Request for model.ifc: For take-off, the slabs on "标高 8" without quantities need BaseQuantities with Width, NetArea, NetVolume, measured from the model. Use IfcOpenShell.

First a look at what the model holds.

```python
import ifcopenshell
import ifcopenshell.util.element
import ifcopenshell.util.unit

model = ifcopenshell.open("model.ifc")
print(model.schema)
for unit_type in ("LENGTHUNIT", "AREAUNIT", "VOLUMEUNIT"):
    print(unit_type, ifcopenshell.util.unit.calculate_unit_scale(model, unit_type))
storey = next(s for s in model.by_type("IfcBuildingStorey") if s.Name == "标高 8")
slabs = [e for e in ifcopenshell.util.element.get_decomposition(storey) if e.is_a("IfcSlab")]
for e in sorted(slabs, key=lambda e: e.id()):
    print(e.id(), e.is_a(), e.Name, list(ifcopenshell.util.element.get_psets(e, qtos_only=True)), sep=" | ")
```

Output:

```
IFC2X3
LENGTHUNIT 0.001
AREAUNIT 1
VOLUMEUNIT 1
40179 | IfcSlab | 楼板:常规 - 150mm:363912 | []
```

```python
import ifcopenshell
import ifcopenshell.api.pset
import ifcopenshell.geom
import ifcopenshell.util.element
import ifcopenshell.util.shape
import ifcopenshell.util.unit

model = ifcopenshell.open("model.ifc")
unit_scale = ifcopenshell.util.unit.calculate_unit_scale(model)
area_scale = ifcopenshell.util.unit.calculate_unit_scale(model, "AREAUNIT")
volume_scale = ifcopenshell.util.unit.calculate_unit_scale(model, "VOLUMEUNIT")
settings = ifcopenshell.geom.settings()

storey = next(s for s in model.by_type("IfcBuildingStorey") if s.Name == "标高 8")
slabs = [e for e in ifcopenshell.util.element.get_decomposition(storey) if e.is_a("IfcSlab")]

for e in sorted(slabs, key=lambda e: e.id()):
    if ifcopenshell.util.element.get_psets(e, qtos_only=True, should_inherit=False):
        continue
    # Geometry comes back in metres, in the element's own axes.
    shape = ifcopenshell.geom.create_shape(settings, e)
    values = {
        "Width": ifcopenshell.util.shape.get_z(shape.geometry) / unit_scale,
        "NetArea": ifcopenshell.util.shape.get_footprint_area(shape.geometry) / area_scale,
        "NetVolume": ifcopenshell.util.shape.get_volume(shape.geometry) / volume_scale,
    }
    qto = ifcopenshell.api.pset.add_qto(model, product=e, name="BaseQuantities")
    ifcopenshell.api.pset.edit_qto(model, qto=qto, properties=values)
    print(e.id(), {k: round(v, 3) for k, v in values.items()})

model.write("model-out.ifc")
```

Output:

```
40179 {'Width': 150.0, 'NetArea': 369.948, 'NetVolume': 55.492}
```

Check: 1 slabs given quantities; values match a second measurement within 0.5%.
